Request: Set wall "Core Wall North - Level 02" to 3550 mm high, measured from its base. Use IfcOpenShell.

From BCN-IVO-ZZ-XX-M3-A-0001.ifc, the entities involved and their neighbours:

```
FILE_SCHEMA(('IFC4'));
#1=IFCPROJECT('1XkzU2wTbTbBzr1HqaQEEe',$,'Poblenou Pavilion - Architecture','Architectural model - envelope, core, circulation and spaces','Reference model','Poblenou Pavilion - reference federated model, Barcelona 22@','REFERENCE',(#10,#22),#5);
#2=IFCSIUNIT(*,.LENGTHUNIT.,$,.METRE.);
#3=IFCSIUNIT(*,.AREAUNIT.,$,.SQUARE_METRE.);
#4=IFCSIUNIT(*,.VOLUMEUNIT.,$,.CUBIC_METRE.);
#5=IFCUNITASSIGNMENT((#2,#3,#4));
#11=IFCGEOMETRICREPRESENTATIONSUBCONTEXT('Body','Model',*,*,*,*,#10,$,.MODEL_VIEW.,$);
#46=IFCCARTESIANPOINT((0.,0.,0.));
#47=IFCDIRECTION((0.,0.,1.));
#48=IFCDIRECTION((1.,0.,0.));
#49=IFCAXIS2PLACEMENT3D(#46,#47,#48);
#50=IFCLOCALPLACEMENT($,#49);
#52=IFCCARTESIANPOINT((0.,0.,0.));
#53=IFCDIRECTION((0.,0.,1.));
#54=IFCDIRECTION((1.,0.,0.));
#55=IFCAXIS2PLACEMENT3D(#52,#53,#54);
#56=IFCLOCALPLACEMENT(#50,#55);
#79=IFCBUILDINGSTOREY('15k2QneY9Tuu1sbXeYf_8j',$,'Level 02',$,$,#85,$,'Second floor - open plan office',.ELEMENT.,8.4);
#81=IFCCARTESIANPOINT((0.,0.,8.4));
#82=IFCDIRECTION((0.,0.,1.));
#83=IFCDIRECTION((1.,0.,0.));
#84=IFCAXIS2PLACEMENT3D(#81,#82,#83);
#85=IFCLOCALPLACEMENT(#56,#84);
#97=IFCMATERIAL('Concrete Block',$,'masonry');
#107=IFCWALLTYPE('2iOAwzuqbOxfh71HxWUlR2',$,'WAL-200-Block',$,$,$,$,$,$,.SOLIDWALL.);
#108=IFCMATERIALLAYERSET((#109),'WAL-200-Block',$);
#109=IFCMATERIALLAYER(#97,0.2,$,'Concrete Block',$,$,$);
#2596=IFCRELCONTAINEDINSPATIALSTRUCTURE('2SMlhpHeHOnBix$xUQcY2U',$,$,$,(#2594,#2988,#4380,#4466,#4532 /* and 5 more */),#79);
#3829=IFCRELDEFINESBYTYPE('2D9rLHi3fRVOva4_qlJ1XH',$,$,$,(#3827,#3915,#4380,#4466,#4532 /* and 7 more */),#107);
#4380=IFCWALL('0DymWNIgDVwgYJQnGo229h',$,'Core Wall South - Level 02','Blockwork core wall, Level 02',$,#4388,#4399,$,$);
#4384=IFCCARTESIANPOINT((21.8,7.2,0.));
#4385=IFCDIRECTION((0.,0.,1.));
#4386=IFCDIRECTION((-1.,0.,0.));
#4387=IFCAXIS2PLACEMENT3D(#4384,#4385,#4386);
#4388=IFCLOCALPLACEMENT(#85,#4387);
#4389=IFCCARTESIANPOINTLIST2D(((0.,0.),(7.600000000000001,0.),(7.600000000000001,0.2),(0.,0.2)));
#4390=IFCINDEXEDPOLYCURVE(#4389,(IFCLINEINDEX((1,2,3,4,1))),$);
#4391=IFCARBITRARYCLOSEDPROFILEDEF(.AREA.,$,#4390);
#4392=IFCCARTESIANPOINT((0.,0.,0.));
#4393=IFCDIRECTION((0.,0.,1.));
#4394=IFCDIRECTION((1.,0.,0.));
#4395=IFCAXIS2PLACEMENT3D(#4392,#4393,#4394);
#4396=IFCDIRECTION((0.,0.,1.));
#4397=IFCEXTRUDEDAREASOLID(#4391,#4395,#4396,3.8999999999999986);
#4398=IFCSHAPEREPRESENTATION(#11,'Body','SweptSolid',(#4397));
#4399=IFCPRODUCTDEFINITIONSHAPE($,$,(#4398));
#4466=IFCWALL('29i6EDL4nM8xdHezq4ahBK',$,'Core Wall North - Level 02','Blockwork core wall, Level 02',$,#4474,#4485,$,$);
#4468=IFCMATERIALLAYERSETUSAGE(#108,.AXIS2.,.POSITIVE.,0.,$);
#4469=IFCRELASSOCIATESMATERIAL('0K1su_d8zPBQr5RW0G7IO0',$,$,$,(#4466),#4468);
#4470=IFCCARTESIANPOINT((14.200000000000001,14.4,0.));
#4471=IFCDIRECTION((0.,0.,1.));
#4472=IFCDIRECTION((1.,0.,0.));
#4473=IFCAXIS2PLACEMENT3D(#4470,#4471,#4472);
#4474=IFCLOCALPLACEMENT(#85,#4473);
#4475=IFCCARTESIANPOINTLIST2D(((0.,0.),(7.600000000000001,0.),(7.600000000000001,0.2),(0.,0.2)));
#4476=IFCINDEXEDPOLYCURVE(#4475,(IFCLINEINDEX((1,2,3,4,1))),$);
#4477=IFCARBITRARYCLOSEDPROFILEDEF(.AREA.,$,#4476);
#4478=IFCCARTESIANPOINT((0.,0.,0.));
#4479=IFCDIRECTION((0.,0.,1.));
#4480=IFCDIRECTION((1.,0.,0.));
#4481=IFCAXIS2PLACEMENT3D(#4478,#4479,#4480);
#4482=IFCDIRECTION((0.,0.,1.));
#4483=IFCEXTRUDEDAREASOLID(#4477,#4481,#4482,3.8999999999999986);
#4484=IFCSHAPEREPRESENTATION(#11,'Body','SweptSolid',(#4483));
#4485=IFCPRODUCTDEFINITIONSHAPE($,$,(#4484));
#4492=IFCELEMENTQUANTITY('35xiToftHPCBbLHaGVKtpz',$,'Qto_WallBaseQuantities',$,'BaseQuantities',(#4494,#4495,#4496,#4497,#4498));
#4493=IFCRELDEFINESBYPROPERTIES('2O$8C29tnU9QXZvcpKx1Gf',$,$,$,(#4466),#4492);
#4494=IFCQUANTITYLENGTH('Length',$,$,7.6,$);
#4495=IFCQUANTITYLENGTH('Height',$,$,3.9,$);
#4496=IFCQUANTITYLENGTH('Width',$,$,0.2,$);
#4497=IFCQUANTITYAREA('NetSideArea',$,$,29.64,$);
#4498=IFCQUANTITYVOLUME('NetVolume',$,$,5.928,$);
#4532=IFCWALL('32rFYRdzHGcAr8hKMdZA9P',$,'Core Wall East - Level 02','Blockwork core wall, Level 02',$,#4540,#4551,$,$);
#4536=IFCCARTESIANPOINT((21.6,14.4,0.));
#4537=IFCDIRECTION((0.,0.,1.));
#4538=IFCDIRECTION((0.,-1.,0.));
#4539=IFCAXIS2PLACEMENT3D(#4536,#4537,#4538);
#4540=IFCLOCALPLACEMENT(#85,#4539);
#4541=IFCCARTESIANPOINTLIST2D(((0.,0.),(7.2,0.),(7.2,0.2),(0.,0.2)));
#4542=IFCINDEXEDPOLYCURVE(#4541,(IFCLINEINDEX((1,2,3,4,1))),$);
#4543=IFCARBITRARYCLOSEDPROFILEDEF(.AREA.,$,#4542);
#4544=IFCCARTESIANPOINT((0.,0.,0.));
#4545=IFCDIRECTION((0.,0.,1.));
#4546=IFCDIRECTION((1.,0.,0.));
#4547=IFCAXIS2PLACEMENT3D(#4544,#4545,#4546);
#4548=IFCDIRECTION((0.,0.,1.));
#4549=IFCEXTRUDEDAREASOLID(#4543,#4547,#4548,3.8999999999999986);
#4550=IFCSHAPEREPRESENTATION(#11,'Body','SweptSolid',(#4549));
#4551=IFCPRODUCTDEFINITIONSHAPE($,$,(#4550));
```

```python
import ifcopenshell
import ifcopenshell.api.pset
import ifcopenshell.geom
import ifcopenshell.util.element
import ifcopenshell.util.representation
import ifcopenshell.util.shape
import ifcopenshell.util.unit

model = ifcopenshell.open("BCN-IVO-ZZ-XX-M3-A-0001.ifc")
area_scale = ifcopenshell.util.unit.calculate_unit_scale(model, "AREAUNIT")
volume_scale = ifcopenshell.util.unit.calculate_unit_scale(model, "VOLUMEUNIT")
settings = ifcopenshell.geom.settings()


def volume(element):
    """Net volume in cubic metres, openings subtracted."""
    shape = ifcopenshell.geom.create_shape(settings, element)
    return ifcopenshell.util.shape.get_volume(shape.geometry)


wall = model.by_guid("29i6EDL4nM8xdHezq4ahBK")
before = volume(wall)

body = ifcopenshell.util.representation.get_representation(wall, "Model", "Body")
solid = body.Items[0]
old_height = solid.Depth
solid.Depth = 3.55
after = volume(wall)
thickness = 0.2  # wall thickness in metres

# Update the stored height, areas and volumes.
qto = model.by_id(ifcopenshell.util.element.get_pset(wall, "Qto_WallBaseQuantities", should_inherit=False)["id"])
ifcopenshell.api.pset.edit_qto(model, qto=qto, properties={
    "Height": solid.Depth,
    "NetSideArea": after / thickness / area_scale,
    "NetVolume": after / volume_scale,
})

print(f"height {old_height:g} -> {solid.Depth:g}, volume {before:.3f} -> {after:.3f} m3")

model.write("BCN-IVO-ZZ-XX-M3-A-0001_edited.ifc")
```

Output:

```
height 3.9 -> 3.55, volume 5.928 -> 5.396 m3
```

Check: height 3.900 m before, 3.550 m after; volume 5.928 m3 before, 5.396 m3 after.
